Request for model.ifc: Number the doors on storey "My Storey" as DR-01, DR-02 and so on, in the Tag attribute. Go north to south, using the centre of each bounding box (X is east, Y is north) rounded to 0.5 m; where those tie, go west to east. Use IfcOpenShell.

First a look at what the model holds.

```python
import ifcopenshell
import ifcopenshell.util.element
import ifcopenshell.util.placement

model = ifcopenshell.open("model.ifc")
print(model.schema)
storey = next(s for s in model.by_type("IfcBuildingStorey") if s.Name == "My Storey")
doors = [e for e in ifcopenshell.util.element.get_decomposition(storey) if e.is_a("IfcDoor")]
for e in sorted(doors, key=lambda e: e.id()):
    origin = ifcopenshell.util.placement.get_local_placement(e.ObjectPlacement)[:3, 3]
    print(e.id(), e.Tag, e.Name, origin.round(2) + 0.0, sep=" | ")
```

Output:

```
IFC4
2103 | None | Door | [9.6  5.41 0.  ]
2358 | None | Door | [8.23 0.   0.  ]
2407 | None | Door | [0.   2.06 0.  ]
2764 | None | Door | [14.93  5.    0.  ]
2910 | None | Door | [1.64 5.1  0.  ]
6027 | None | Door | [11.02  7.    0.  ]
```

```python
import ifcopenshell
import ifcopenshell.geom
import ifcopenshell.util.element
import ifcopenshell.util.shape

model = ifcopenshell.open("model.ifc")
settings = ifcopenshell.geom.settings()
settings.set("use-world-coords", True)


def centre(element):
    shape = ifcopenshell.geom.create_shape(settings, element)
    return ifcopenshell.util.shape.get_bbox_centroid(shape.geometry)


storey = next(s for s in model.by_type("IfcBuildingStorey") if s.Name == "My Storey")
doors = [e for e in ifcopenshell.util.element.get_decomposition(storey) if e.is_a("IfcDoor")]

# Insertion points can sit at a corner or the storey origin, so sort by the geometry (in metres).
centres = {e: centre(e) for e in doors}
doors.sort(key=lambda e: (-round(centres[e][1] / 0.5), centres[e][0]))

for i, e in enumerate(doors, start=1):
    number = f"DR-{i:02d}"
    e.Tag = number
    print(e.id(), number)

model.write("model_v2.ifc")
```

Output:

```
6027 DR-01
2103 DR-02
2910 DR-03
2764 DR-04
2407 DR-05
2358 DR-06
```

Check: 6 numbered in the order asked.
